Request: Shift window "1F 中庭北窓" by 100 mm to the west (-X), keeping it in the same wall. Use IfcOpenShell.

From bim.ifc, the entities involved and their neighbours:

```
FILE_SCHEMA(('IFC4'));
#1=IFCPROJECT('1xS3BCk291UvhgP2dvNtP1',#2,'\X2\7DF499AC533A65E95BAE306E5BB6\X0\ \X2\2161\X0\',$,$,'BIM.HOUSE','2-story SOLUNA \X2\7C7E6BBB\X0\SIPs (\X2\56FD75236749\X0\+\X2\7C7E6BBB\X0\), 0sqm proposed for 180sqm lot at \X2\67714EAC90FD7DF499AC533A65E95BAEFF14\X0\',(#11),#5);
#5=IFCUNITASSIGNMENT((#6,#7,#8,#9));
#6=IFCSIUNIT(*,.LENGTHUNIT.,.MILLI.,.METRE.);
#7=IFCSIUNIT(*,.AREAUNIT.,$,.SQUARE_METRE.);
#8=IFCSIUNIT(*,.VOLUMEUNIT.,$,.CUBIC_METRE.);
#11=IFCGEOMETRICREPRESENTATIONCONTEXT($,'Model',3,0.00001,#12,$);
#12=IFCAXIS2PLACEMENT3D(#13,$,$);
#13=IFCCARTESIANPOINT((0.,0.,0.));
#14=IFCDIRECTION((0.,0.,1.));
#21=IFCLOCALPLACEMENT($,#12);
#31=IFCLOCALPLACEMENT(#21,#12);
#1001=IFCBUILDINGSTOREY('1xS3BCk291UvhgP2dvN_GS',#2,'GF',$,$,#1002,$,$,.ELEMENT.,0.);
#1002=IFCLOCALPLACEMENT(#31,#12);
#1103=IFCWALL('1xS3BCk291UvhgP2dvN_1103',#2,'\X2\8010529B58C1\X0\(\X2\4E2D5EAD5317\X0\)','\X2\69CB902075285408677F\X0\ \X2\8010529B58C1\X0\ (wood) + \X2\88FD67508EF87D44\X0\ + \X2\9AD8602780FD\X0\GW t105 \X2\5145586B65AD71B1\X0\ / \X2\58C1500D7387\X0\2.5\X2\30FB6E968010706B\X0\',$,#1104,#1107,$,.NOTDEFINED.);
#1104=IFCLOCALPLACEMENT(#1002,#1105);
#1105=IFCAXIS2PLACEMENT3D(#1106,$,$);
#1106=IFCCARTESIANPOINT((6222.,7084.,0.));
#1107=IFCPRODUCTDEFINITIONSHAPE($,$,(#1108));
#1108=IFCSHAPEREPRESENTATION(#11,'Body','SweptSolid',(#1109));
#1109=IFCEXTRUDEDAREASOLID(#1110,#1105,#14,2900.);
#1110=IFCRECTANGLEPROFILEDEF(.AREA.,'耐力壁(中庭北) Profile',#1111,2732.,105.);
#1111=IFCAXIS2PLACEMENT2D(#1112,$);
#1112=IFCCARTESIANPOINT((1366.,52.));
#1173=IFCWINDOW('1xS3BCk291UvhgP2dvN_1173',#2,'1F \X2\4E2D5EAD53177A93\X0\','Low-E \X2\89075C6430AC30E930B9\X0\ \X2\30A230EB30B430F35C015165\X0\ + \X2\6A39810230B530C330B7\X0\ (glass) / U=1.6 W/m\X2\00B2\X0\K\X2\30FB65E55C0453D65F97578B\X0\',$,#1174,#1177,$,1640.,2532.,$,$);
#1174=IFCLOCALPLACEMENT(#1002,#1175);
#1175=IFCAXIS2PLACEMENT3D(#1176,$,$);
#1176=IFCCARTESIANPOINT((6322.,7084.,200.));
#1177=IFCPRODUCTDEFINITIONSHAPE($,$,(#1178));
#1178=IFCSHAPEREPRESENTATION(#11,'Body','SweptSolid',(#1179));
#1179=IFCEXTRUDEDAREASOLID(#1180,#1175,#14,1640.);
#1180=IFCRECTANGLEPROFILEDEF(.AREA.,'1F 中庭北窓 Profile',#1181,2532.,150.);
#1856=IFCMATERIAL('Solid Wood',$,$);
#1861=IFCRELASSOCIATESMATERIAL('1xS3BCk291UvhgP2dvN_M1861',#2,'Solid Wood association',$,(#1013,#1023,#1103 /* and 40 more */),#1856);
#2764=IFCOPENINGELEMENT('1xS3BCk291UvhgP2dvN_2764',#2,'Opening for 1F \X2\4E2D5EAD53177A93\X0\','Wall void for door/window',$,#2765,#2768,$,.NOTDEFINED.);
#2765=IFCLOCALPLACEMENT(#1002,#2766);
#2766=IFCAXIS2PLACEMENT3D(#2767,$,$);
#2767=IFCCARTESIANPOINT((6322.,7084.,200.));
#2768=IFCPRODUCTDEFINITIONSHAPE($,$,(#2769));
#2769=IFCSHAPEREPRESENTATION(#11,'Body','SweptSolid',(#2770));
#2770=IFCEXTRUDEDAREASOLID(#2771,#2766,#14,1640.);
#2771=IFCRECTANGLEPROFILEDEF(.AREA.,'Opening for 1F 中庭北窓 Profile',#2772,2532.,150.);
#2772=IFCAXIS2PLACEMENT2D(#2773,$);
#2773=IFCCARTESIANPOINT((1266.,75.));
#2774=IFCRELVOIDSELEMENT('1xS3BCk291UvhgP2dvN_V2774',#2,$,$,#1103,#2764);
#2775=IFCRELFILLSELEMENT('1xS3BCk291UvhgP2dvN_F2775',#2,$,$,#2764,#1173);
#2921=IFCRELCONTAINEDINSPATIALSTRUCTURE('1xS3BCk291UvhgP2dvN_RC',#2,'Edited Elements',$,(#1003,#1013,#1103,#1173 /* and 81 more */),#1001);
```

```python
import ifcopenshell
import ifcopenshell.api.geometry
import ifcopenshell.util.placement

model = ifcopenshell.open("bim.ifc")

window = model.by_guid("1xS3BCk291UvhgP2dvN_1173")
opening = window.FillsVoids[0].RelatingOpeningElement
wall = opening.VoidsElements[0].RelatingBuildingElement

wall_matrix = ifcopenshell.util.placement.get_local_placement(wall.ObjectPlacement)
shift = wall_matrix[:3, 0] * -100.0
before = ifcopenshell.util.placement.get_local_placement(window.ObjectPlacement)[:3, 3].copy()

# The window is not placed relative to its opening, so move both.
for product in (opening, window):
    matrix = ifcopenshell.util.placement.get_local_placement(product.ObjectPlacement)
    matrix[:3, 3] += shift
    ifcopenshell.api.geometry.edit_object_placement(model, product=product, matrix=matrix, is_si=False)

after = ifcopenshell.util.placement.get_local_placement(window.ObjectPlacement)[:3, 3]
print("window moved by", (after - before).round(3) + 0.0)

model.write("bim_updated.ifc")
```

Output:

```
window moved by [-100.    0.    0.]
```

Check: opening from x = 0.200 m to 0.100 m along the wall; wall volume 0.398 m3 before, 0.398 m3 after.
